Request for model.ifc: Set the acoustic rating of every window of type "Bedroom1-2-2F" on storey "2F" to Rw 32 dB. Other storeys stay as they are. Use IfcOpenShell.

First a look at what the model holds.

```python
import ifcopenshell
import ifcopenshell.util.element

model = ifcopenshell.open("model.ifc")
print(model.schema)
storey = next(s for s in model.by_type("IfcBuildingStorey") if s.Name == "2F")
windows = [e for e in ifcopenshell.util.element.get_decomposition(storey) if e.is_a("IfcWindow")]
seen = {}
for e in windows:
    element_type = ifcopenshell.util.element.get_type(e)
    key = (element_type.Name if element_type != e and element_type else None, ifcopenshell.util.element.get_pset(e, "Pset_WindowCommon", "AcousticRating"))
    seen[key] = seen.get(key, 0) + 1
for (name, value), count in sorted(seen.items(), key=str):
    print(count, "x", name, "|", value)
```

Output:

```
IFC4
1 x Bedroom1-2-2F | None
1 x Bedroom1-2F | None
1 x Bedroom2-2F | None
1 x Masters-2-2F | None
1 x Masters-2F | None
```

```python
import ifcopenshell
import ifcopenshell.api.pset
import ifcopenshell.util.element

model = ifcopenshell.open("model.ifc")

storey = next(s for s in model.by_type("IfcBuildingStorey") if s.Name == "2F")
windows = [e for e in ifcopenshell.util.element.get_decomposition(storey) if e.is_a("IfcWindow")]

count = 0
for e in windows:
    element_type = ifcopenshell.util.element.get_type(e)
    if element_type in (None, e) or element_type.Name != "Bedroom1-2-2F":
        continue
    # add_pset returns the element's existing set when there is one.
    pset = ifcopenshell.api.pset.add_pset(model, product=e, name="Pset_WindowCommon")
    ifcopenshell.api.pset.edit_pset(model, pset=pset, properties={"AcousticRating": "Rw 32 dB"})
    count += 1

print(count, "windows updated")

model.write("model_updated.ifc")
```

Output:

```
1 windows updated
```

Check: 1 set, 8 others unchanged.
